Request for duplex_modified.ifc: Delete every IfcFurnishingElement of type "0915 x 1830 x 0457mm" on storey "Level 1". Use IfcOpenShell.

First a look at what the model holds.

```python
import ifcopenshell
import ifcopenshell.util.element

model = ifcopenshell.open("duplex_modified.ifc")
print(model.schema)
storey = next(s for s in model.by_type("IfcBuildingStorey") if s.Name == "Level 1")
furniture = [e for e in ifcopenshell.util.element.get_decomposition(storey) if e.is_a("IfcFurnishingElement")]
seen = {}
for e in furniture:
    element_type = ifcopenshell.util.element.get_type(e)
    name = element_type.Name if element_type not in (None, e) else None
    seen[name] = seen.get(name, 0) + 1
for name, count in sorted(seen.items(), key=str):
    print(count, "x", name)
```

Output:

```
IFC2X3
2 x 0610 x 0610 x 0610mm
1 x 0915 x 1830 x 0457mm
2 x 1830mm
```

```python
import ifcopenshell
import ifcopenshell.api.root
import ifcopenshell.util.element

model = ifcopenshell.open("duplex_modified.ifc")

storey = next(s for s in model.by_type("IfcBuildingStorey") if s.Name == "Level 1")
furniture = [e for e in ifcopenshell.util.element.get_decomposition(storey) if e.is_a("IfcFurnishingElement")]
targets = [e for e in furniture if (t := ifcopenshell.util.element.get_type(e)) not in (None, e) and t.Name == "0915 x 1830 x 0457mm"]

for e in targets:
    ifcopenshell.api.root.remove_product(model, product=e)
print(len(targets), "removed")

model.write("duplex_modified_v2.ifc")
```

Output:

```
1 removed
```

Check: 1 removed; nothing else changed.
